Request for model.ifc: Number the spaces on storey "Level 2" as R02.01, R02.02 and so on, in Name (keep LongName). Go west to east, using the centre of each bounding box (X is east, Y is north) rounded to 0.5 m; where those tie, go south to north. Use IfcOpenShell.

First a look at what the model holds.

```python
import ifcopenshell
import ifcopenshell.util.element
import ifcopenshell.util.placement

model = ifcopenshell.open("model.ifc")
print(model.schema)
storey = next(s for s in model.by_type("IfcBuildingStorey") if s.Name == "Level 2")
spaces = [e for e in ifcopenshell.util.element.get_decomposition(storey) if e.is_a("IfcSpace")]
for e in sorted(spaces, key=lambda e: e.id()):
    origin = ifcopenshell.util.placement.get_local_placement(e.ObjectPlacement)[:3, 3]
    print(e.id(), e.Name, e.LongName, origin.round(2) + 0.0, sep=" | ")
```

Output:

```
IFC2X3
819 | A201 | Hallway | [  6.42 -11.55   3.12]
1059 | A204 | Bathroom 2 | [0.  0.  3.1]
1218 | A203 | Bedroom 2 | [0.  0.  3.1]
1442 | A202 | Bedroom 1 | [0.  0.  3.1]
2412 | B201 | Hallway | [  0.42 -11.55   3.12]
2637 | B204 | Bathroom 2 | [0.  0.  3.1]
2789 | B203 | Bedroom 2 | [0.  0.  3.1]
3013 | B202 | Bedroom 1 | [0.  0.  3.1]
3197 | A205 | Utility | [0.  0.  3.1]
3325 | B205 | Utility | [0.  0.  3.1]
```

```python
import ifcopenshell
import ifcopenshell.geom
import ifcopenshell.util.element
import ifcopenshell.util.shape

model = ifcopenshell.open("model.ifc")
settings = ifcopenshell.geom.settings()
settings.set("use-world-coords", True)


def centre(element):
    shape = ifcopenshell.geom.create_shape(settings, element)
    return ifcopenshell.util.shape.get_bbox_centroid(shape.geometry)


storey = next(s for s in model.by_type("IfcBuildingStorey") if s.Name == "Level 2")
spaces = [e for e in ifcopenshell.util.element.get_decomposition(storey) if e.is_a("IfcSpace")]

# Insertion points can sit at a corner or the storey origin, so sort by the geometry (in metres).
centres = {e: centre(e) for e in spaces}
spaces.sort(key=lambda e: (round(centres[e][0] / 0.5), centres[e][1]))

for i, e in enumerate(spaces, start=1):
    number = f"R02.{i:02d}"
    e.Name = number
    print(e.id(), number)

model.write("model_v2.ifc")
```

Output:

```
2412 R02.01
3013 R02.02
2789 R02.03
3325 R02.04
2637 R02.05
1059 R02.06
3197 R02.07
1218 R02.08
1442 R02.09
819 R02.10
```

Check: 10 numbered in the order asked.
